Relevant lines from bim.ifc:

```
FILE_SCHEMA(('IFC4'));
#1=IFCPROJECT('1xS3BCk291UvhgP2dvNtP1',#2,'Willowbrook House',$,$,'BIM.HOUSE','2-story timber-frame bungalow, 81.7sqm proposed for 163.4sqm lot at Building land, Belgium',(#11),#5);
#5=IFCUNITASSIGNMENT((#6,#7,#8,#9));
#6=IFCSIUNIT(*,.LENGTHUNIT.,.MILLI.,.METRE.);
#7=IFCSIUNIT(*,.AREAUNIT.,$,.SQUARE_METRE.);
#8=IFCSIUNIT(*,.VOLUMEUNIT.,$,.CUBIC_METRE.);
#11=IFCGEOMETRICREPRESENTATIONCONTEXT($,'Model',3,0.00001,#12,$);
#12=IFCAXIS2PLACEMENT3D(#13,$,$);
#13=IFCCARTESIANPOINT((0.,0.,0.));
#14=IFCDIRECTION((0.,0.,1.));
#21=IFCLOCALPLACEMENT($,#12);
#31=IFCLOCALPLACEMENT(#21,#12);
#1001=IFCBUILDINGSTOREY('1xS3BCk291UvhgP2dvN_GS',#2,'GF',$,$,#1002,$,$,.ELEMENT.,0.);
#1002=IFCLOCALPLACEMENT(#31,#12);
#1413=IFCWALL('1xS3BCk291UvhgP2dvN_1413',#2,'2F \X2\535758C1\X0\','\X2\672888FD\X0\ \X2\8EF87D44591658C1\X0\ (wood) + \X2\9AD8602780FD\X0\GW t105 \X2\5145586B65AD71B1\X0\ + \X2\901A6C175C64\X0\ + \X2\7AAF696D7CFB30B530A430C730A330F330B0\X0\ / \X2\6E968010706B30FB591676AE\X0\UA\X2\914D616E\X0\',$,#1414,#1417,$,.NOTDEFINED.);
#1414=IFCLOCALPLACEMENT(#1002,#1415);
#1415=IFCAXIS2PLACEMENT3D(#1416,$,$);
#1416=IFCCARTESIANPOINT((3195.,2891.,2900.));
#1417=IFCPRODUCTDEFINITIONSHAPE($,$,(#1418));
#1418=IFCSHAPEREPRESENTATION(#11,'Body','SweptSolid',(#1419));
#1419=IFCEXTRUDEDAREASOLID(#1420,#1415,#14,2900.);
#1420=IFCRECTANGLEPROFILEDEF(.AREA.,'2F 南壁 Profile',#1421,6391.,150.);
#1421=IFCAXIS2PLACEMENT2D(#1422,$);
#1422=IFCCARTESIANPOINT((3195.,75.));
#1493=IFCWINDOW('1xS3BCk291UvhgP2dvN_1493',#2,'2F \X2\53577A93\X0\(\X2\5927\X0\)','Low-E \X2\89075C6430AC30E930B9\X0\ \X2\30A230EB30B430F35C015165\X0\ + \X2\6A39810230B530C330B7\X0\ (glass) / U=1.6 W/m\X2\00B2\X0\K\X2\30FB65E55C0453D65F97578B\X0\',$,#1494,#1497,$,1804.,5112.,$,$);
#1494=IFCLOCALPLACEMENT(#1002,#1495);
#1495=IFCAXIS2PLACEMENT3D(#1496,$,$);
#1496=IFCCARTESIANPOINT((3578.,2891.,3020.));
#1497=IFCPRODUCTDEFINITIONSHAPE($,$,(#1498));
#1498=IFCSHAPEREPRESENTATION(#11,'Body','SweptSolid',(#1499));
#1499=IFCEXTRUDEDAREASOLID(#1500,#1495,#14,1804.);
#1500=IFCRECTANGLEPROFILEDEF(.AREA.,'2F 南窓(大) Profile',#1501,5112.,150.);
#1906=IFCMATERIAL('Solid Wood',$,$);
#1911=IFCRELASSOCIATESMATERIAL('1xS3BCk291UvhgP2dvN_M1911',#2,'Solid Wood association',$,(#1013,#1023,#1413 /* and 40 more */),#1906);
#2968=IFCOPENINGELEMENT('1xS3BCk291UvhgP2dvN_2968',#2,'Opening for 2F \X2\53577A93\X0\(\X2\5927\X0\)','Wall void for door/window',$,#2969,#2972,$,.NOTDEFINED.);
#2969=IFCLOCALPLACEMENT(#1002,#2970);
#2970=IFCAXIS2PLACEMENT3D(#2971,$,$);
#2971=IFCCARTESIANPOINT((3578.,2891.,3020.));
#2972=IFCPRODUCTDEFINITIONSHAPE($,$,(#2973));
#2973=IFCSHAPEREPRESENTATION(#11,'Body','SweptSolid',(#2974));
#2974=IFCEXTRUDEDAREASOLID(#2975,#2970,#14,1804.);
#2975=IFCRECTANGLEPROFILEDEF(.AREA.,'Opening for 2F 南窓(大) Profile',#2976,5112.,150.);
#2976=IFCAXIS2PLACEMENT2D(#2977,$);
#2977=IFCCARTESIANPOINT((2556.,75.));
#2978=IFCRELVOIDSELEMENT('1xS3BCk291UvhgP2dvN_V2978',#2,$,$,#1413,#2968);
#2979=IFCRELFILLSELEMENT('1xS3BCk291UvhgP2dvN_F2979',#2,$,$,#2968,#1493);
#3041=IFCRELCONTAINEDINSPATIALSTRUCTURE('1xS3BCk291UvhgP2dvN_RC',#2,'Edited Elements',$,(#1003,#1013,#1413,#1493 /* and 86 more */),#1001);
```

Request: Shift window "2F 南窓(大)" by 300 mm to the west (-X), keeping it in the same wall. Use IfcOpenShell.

```python
import ifcopenshell
import ifcopenshell.api.geometry
import ifcopenshell.util.placement
import ifcopenshell.util.unit

model = ifcopenshell.open("bim.ifc")
unit_scale = ifcopenshell.util.unit.calculate_unit_scale(model)

window = model.by_guid("1xS3BCk291UvhgP2dvN_1493")
opening = window.FillsVoids[0].RelatingOpeningElement
wall = opening.VoidsElements[0].RelatingBuildingElement

wall_matrix = ifcopenshell.util.placement.get_local_placement(wall.ObjectPlacement)
shift = wall_matrix[:3, 0] * -0.3 / unit_scale
before = ifcopenshell.util.placement.get_local_placement(window.ObjectPlacement)[:3, 3].copy()

# The window is not placed relative to its opening, so move both.
for product in (opening, window):
    matrix = ifcopenshell.util.placement.get_local_placement(product.ObjectPlacement)
    matrix[:3, 3] += shift
    ifcopenshell.api.geometry.edit_object_placement(model, product=product, matrix=matrix, is_si=False)

after = ifcopenshell.util.placement.get_local_placement(window.ObjectPlacement)[:3, 3]
print("window moved by", (after - before).round(3) + 0.0)

model.write("bim_rev.ifc")
```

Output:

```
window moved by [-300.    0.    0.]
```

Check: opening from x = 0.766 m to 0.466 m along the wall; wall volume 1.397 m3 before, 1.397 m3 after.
